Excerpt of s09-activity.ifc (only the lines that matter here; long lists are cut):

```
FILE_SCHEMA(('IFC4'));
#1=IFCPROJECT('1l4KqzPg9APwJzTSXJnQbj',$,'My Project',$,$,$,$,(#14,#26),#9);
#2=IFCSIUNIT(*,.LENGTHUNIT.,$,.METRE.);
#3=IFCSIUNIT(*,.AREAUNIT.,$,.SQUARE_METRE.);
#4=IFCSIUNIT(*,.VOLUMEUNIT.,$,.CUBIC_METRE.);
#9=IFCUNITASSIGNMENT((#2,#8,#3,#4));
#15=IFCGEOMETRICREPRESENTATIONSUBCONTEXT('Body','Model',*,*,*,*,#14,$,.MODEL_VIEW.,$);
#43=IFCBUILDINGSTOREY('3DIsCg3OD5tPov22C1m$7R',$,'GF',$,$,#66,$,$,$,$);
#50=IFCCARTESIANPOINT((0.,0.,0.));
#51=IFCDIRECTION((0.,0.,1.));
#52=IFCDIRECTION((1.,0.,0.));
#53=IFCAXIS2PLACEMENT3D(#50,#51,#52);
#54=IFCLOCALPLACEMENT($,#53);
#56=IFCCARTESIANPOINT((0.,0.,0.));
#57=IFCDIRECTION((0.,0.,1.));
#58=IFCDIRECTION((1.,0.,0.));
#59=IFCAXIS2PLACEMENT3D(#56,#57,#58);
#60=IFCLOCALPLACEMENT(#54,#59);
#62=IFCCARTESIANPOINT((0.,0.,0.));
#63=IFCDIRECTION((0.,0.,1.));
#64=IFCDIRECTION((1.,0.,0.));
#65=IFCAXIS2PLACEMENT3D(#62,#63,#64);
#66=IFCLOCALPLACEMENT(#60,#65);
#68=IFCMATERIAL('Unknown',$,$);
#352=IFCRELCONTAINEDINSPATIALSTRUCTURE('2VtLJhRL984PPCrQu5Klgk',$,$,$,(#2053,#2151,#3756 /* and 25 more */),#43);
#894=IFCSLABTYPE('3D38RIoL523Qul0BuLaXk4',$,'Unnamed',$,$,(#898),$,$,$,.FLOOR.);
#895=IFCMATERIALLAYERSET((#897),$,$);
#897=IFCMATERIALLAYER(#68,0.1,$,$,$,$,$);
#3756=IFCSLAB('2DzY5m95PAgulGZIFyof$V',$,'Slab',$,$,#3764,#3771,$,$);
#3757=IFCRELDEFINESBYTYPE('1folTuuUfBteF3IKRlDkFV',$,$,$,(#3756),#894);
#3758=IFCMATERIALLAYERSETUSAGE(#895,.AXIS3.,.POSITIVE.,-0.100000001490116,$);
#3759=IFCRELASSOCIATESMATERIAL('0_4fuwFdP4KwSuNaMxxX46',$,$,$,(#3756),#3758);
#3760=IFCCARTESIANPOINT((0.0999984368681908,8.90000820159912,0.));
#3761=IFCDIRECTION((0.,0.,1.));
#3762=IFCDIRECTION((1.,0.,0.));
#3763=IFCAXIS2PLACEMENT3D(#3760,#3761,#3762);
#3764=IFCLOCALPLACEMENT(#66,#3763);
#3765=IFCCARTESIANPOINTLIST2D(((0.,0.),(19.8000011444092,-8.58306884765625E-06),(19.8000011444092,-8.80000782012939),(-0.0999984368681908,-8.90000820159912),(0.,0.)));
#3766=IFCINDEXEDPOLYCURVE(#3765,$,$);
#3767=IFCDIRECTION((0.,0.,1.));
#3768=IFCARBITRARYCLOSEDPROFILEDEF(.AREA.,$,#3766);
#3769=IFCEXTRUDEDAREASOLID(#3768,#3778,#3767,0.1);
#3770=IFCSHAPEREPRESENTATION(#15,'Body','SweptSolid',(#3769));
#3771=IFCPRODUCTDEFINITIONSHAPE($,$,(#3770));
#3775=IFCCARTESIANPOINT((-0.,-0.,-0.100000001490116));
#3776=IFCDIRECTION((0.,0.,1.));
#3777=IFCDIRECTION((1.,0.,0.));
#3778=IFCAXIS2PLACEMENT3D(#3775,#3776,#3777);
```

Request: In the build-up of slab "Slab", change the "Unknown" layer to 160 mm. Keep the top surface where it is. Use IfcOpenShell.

```python
import ifcopenshell
import ifcopenshell.util.element
import ifcopenshell.util.representation

model = ifcopenshell.open("s09-activity.ifc")

layer_set = model.by_id(895)
layer = next(l for l in layer_set.MaterialLayers if l.Material and l.Material.Name == "Unknown")
change = 0.16 - layer.LayerThickness
layer.LayerThickness += change

# Geometry does not follow the layer set by itself.
slabs = [e for e in ifcopenshell.util.element.get_elements_by_material(model, layer_set) if e.is_a("IfcSlab")]
for slab in sorted(slabs, key=lambda e: e.id()):
    body = ifcopenshell.util.representation.get_representation(slab, "Model", "Body")
    solid = body.Items[0]
    old_depth = solid.Depth
    solid.Depth += change
    # Extruded upwards: lower the start of the extrusion so the top stays.
    x, y, z = solid.Position.Location.Coordinates
    solid.Position.Location = model.createIfcCartesianPoint((x, y, z - change))
    print(slab.id(), f"{old_depth:g} -> {solid.Depth:g}")

# The layers are counted up from the underside, which has moved.
for usage in {ifcopenshell.util.element.get_material(slab) for slab in slabs}:
    usage.OffsetFromReferenceLine -= change

model.write("s09-activity_v2.ifc")
```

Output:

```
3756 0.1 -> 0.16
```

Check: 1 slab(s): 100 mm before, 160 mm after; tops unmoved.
